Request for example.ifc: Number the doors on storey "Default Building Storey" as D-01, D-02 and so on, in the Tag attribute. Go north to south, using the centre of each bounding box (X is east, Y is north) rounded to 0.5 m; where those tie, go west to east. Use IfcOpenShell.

First a look at what the model holds.

```python
import ifcopenshell
import ifcopenshell.util.element
import ifcopenshell.util.placement

model = ifcopenshell.open("example.ifc")
print(model.schema)
storey = next(s for s in model.by_type("IfcBuildingStorey") if s.Name == "Default Building Storey")
doors = [e for e in ifcopenshell.util.element.get_decomposition(storey) if e.is_a("IfcDoor")]
for e in sorted(doors, key=lambda e: e.id()):
    origin = ifcopenshell.util.placement.get_local_placement(e.ObjectPlacement)[:3, 3]
    print(e.id(), e.Tag, e.Name, origin.round(2) + 0.0, sep=" | ")
```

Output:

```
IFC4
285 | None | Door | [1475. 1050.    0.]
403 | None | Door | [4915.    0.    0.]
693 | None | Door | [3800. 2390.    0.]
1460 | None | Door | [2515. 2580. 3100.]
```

```python
import ifcopenshell
import ifcopenshell.geom
import ifcopenshell.util.element
import ifcopenshell.util.shape

model = ifcopenshell.open("example.ifc")
settings = ifcopenshell.geom.settings()
settings.set("use-world-coords", True)


def centre(element):
    shape = ifcopenshell.geom.create_shape(settings, element)
    return ifcopenshell.util.shape.get_bbox_centroid(shape.geometry)


storey = next(s for s in model.by_type("IfcBuildingStorey") if s.Name == "Default Building Storey")
doors = [e for e in ifcopenshell.util.element.get_decomposition(storey) if e.is_a("IfcDoor")]

# Insertion points can sit at a corner or the storey origin, so sort by the geometry (in metres).
centres = {e: centre(e) for e in doors}
doors.sort(key=lambda e: (-round(centres[e][1] / 0.5), centres[e][0]))

for i, e in enumerate(doors, start=1):
    number = f"D-{i:02d}"
    e.Tag = number
    print(e.id(), number)

model.write("example_v2.ifc")
```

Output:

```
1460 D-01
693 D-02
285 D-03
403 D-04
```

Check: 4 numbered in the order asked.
